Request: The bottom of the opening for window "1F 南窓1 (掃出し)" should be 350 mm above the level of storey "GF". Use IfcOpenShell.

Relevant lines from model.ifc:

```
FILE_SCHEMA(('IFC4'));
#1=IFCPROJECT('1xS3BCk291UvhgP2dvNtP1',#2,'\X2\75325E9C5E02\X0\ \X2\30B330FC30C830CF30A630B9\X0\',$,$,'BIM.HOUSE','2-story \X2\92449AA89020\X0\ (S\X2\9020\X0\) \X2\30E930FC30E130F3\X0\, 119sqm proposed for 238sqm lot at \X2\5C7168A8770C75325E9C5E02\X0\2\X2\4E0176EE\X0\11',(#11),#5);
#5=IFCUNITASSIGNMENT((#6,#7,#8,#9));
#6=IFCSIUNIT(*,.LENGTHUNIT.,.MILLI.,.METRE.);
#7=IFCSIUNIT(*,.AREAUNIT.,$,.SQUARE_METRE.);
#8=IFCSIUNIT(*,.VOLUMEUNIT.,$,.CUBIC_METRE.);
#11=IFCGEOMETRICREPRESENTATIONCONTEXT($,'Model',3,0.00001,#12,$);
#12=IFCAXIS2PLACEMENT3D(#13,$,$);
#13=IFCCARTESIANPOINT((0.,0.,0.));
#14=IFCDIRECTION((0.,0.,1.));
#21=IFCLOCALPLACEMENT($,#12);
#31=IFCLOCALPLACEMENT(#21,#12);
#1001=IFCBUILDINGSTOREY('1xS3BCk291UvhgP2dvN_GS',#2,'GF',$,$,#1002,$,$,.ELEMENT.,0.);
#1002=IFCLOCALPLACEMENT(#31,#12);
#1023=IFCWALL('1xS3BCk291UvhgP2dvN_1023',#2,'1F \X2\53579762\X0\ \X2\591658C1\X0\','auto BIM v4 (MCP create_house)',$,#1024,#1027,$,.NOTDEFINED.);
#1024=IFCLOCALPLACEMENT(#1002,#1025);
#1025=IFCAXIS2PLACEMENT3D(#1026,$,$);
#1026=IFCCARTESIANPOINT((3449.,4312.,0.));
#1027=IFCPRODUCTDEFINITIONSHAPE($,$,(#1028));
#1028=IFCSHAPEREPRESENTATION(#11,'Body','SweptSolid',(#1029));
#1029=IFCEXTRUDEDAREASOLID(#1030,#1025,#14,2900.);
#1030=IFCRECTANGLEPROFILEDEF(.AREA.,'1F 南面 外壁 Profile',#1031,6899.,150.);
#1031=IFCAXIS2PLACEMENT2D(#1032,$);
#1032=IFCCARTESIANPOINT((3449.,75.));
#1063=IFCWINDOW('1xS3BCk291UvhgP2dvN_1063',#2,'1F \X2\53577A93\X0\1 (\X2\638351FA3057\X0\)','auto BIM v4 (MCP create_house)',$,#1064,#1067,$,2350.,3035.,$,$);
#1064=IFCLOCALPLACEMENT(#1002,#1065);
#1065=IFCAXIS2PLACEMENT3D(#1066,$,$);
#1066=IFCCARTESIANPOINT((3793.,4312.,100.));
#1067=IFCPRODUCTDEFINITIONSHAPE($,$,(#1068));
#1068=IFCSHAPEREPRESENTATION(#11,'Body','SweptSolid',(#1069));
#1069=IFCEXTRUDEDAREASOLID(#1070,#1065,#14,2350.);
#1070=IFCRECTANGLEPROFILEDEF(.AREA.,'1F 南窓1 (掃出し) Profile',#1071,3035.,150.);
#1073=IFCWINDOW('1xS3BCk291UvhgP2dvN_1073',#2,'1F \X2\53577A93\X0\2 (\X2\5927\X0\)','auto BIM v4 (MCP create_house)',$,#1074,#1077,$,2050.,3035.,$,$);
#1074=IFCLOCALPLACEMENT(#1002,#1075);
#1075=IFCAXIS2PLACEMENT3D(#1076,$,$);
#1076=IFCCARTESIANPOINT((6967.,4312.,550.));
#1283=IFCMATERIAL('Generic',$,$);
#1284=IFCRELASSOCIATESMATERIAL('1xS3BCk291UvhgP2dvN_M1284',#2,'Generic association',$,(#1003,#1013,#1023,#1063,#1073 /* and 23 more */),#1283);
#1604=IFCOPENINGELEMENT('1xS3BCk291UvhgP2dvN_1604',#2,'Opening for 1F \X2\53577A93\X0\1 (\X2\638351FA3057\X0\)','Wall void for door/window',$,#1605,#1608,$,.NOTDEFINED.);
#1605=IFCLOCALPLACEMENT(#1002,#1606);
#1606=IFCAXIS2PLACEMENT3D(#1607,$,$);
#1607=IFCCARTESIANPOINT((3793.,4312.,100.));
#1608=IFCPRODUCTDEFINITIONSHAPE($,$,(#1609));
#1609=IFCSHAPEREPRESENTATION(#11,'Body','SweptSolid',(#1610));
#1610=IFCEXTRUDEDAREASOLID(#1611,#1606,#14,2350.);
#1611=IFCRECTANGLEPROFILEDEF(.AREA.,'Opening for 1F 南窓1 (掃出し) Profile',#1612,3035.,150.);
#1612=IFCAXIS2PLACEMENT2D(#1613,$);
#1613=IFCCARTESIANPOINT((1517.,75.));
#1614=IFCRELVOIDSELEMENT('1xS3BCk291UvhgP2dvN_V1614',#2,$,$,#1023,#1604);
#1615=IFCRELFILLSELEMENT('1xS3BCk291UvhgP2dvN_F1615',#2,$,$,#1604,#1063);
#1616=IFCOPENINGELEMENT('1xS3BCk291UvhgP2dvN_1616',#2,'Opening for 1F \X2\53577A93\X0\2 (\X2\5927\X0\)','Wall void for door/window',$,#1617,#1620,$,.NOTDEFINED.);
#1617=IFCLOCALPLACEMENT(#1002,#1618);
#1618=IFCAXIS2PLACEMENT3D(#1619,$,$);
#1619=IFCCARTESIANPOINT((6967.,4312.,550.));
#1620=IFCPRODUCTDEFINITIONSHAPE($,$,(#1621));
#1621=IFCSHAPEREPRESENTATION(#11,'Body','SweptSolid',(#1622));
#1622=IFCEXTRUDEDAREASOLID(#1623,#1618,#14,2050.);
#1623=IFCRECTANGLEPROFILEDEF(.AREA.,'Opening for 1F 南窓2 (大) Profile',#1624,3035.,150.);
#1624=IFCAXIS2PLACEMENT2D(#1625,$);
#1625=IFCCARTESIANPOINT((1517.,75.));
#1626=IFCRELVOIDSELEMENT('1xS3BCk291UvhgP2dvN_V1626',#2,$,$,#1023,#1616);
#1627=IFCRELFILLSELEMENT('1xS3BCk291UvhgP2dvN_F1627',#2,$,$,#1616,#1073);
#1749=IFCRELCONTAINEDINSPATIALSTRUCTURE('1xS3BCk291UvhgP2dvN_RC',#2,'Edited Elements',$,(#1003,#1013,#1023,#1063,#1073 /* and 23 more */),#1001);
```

```python
import numpy as np
import ifcopenshell
import ifcopenshell.api.geometry
import ifcopenshell.geom
import ifcopenshell.util.element
import ifcopenshell.util.placement
import ifcopenshell.util.shape
import ifcopenshell.util.unit

model = ifcopenshell.open("model.ifc")
unit_scale = ifcopenshell.util.unit.calculate_unit_scale(model)

window = model.by_id(1063)
opening = window.FillsVoids[0].RelatingOpeningElement
storey = ifcopenshell.util.element.get_container(window, ifc_class="IfcBuildingStorey")
level = ifcopenshell.util.placement.get_local_placement(storey.ObjectPlacement)[2, 3]

# The opening's origin need not be at the sill, so measure its lowest point.
shape = ifcopenshell.geom.create_shape(ifcopenshell.geom.settings(), opening)
bottom = ifcopenshell.util.shape.get_shape_bottom_elevation(shape, shape.geometry) / unit_scale
dz = level + 0.35 / unit_scale - bottom

shift = np.array([0.0, 0.0, dz])
# The window is not placed relative to its opening, so move both.
for product in (opening, window):
    matrix = ifcopenshell.util.placement.get_local_placement(product.ObjectPlacement)
    matrix[:3, 3] += shift
    ifcopenshell.api.geometry.edit_object_placement(model, product=product, matrix=matrix, is_si=False)

print(f"moved by {dz * unit_scale:+.3f} m")

model.write("model_updated.ifc")
```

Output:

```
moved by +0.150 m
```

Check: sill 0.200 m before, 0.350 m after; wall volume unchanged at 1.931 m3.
